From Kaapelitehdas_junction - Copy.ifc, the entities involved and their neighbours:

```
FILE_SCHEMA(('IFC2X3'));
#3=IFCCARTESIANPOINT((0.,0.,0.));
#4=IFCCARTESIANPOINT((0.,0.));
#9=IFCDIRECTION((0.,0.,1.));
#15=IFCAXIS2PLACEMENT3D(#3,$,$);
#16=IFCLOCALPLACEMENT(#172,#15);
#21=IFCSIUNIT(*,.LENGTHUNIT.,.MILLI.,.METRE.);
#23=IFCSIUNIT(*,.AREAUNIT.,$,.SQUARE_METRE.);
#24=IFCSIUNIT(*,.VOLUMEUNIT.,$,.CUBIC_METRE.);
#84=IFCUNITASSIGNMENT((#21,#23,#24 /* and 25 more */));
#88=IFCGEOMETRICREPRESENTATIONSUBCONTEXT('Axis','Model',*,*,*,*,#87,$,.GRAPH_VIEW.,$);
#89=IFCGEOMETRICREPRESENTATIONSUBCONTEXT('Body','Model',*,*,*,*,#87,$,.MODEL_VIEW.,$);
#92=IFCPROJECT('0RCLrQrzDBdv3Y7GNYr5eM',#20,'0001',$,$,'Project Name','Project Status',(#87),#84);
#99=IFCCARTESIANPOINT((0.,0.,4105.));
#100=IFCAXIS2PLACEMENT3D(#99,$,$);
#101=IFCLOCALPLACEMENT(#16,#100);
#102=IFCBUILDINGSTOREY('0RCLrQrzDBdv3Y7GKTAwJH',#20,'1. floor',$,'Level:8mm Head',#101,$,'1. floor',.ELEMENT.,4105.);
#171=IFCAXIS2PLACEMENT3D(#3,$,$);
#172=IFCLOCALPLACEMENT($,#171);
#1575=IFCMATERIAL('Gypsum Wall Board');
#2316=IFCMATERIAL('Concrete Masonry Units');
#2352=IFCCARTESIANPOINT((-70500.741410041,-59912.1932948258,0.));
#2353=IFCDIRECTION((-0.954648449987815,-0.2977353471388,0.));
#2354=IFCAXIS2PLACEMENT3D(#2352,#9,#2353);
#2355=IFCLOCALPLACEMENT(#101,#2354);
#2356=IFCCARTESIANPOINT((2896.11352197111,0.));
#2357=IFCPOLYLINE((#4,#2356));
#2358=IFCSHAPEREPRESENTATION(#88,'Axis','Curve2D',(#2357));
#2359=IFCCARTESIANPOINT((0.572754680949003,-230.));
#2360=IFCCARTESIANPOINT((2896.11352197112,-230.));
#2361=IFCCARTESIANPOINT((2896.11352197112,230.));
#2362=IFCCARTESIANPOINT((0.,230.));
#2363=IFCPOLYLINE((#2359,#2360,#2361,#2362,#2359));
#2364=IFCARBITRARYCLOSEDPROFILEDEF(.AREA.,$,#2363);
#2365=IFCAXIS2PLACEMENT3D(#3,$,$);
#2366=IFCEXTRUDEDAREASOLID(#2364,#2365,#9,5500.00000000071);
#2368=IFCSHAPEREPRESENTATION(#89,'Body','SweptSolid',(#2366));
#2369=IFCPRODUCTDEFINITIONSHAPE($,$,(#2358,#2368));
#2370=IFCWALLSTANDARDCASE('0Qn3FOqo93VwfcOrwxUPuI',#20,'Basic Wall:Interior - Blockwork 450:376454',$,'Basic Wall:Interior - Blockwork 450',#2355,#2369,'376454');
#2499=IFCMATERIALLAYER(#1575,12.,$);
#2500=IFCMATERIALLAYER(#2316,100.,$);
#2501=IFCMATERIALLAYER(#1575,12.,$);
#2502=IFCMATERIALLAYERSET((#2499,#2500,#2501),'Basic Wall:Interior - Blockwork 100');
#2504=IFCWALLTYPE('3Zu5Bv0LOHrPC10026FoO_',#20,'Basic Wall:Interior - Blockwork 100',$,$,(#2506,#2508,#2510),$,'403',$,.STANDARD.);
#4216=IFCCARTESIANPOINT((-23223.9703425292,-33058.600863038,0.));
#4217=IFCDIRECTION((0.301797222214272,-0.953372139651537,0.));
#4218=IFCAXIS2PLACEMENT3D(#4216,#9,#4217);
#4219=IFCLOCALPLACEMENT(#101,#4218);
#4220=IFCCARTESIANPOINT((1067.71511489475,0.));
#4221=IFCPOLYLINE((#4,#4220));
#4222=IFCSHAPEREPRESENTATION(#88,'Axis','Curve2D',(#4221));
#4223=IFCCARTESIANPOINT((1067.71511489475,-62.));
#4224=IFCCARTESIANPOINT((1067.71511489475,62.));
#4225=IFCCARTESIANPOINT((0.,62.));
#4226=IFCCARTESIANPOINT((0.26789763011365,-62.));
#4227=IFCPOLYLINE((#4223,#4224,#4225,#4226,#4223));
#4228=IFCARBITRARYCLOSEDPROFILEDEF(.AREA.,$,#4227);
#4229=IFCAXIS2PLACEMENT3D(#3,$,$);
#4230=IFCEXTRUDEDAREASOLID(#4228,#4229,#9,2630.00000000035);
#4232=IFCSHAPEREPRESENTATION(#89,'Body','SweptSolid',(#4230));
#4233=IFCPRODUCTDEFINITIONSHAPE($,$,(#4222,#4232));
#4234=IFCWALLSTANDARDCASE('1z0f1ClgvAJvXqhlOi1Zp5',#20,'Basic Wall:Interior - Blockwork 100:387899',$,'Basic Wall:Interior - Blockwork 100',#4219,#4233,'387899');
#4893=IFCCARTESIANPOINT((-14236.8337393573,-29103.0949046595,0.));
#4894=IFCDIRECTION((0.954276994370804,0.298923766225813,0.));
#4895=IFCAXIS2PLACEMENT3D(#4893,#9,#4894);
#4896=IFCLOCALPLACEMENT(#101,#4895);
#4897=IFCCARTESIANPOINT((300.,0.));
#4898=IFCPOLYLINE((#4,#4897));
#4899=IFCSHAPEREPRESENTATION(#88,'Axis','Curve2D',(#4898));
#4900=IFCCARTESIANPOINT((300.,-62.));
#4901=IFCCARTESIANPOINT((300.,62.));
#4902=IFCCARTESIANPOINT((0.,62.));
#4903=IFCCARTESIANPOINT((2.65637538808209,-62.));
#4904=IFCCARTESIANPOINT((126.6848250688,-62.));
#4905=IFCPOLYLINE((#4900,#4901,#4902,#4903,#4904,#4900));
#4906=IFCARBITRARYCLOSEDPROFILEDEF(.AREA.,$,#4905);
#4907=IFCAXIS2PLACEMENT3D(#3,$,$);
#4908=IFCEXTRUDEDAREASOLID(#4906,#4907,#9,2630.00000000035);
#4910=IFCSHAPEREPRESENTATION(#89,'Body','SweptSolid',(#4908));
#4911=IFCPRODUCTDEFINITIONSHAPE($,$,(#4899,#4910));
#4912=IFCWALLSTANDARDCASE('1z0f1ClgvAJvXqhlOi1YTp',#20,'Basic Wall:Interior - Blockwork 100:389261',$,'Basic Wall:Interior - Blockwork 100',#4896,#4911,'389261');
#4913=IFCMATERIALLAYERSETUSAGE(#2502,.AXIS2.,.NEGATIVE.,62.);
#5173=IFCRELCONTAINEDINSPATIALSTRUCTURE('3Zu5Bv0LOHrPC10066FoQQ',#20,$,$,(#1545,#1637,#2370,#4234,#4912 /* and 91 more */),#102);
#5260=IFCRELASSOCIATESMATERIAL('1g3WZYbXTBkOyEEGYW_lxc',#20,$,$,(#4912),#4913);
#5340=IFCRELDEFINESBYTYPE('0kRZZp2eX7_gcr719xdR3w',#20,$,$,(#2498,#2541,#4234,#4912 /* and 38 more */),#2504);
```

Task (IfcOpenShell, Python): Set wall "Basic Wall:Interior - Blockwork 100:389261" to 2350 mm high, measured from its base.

```python
import ifcopenshell
import ifcopenshell.geom
import ifcopenshell.util.representation
import ifcopenshell.util.shape
import ifcopenshell.util.unit

model = ifcopenshell.open("Kaapelitehdas_junction - Copy.ifc")
unit_scale = ifcopenshell.util.unit.calculate_unit_scale(model)
settings = ifcopenshell.geom.settings()


def volume(element):
    """Net volume in cubic metres, openings subtracted."""
    shape = ifcopenshell.geom.create_shape(settings, element)
    return ifcopenshell.util.shape.get_volume(shape.geometry)


wall = model.by_guid("1z0f1ClgvAJvXqhlOi1YTp")
before = volume(wall)

body = ifcopenshell.util.representation.get_representation(wall, "Model", "Body")
solid = body.Items[0]
old_height = solid.Depth
solid.Depth = 2.35 / unit_scale
after = volume(wall)

print(f"height {old_height:g} -> {solid.Depth:g}, volume {before:.3f} -> {after:.3f} m3")

model.write("Kaapelitehdas_junction - Copy_updated.ifc")
```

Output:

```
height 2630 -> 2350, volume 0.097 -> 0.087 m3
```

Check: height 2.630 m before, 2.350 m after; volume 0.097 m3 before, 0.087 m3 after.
